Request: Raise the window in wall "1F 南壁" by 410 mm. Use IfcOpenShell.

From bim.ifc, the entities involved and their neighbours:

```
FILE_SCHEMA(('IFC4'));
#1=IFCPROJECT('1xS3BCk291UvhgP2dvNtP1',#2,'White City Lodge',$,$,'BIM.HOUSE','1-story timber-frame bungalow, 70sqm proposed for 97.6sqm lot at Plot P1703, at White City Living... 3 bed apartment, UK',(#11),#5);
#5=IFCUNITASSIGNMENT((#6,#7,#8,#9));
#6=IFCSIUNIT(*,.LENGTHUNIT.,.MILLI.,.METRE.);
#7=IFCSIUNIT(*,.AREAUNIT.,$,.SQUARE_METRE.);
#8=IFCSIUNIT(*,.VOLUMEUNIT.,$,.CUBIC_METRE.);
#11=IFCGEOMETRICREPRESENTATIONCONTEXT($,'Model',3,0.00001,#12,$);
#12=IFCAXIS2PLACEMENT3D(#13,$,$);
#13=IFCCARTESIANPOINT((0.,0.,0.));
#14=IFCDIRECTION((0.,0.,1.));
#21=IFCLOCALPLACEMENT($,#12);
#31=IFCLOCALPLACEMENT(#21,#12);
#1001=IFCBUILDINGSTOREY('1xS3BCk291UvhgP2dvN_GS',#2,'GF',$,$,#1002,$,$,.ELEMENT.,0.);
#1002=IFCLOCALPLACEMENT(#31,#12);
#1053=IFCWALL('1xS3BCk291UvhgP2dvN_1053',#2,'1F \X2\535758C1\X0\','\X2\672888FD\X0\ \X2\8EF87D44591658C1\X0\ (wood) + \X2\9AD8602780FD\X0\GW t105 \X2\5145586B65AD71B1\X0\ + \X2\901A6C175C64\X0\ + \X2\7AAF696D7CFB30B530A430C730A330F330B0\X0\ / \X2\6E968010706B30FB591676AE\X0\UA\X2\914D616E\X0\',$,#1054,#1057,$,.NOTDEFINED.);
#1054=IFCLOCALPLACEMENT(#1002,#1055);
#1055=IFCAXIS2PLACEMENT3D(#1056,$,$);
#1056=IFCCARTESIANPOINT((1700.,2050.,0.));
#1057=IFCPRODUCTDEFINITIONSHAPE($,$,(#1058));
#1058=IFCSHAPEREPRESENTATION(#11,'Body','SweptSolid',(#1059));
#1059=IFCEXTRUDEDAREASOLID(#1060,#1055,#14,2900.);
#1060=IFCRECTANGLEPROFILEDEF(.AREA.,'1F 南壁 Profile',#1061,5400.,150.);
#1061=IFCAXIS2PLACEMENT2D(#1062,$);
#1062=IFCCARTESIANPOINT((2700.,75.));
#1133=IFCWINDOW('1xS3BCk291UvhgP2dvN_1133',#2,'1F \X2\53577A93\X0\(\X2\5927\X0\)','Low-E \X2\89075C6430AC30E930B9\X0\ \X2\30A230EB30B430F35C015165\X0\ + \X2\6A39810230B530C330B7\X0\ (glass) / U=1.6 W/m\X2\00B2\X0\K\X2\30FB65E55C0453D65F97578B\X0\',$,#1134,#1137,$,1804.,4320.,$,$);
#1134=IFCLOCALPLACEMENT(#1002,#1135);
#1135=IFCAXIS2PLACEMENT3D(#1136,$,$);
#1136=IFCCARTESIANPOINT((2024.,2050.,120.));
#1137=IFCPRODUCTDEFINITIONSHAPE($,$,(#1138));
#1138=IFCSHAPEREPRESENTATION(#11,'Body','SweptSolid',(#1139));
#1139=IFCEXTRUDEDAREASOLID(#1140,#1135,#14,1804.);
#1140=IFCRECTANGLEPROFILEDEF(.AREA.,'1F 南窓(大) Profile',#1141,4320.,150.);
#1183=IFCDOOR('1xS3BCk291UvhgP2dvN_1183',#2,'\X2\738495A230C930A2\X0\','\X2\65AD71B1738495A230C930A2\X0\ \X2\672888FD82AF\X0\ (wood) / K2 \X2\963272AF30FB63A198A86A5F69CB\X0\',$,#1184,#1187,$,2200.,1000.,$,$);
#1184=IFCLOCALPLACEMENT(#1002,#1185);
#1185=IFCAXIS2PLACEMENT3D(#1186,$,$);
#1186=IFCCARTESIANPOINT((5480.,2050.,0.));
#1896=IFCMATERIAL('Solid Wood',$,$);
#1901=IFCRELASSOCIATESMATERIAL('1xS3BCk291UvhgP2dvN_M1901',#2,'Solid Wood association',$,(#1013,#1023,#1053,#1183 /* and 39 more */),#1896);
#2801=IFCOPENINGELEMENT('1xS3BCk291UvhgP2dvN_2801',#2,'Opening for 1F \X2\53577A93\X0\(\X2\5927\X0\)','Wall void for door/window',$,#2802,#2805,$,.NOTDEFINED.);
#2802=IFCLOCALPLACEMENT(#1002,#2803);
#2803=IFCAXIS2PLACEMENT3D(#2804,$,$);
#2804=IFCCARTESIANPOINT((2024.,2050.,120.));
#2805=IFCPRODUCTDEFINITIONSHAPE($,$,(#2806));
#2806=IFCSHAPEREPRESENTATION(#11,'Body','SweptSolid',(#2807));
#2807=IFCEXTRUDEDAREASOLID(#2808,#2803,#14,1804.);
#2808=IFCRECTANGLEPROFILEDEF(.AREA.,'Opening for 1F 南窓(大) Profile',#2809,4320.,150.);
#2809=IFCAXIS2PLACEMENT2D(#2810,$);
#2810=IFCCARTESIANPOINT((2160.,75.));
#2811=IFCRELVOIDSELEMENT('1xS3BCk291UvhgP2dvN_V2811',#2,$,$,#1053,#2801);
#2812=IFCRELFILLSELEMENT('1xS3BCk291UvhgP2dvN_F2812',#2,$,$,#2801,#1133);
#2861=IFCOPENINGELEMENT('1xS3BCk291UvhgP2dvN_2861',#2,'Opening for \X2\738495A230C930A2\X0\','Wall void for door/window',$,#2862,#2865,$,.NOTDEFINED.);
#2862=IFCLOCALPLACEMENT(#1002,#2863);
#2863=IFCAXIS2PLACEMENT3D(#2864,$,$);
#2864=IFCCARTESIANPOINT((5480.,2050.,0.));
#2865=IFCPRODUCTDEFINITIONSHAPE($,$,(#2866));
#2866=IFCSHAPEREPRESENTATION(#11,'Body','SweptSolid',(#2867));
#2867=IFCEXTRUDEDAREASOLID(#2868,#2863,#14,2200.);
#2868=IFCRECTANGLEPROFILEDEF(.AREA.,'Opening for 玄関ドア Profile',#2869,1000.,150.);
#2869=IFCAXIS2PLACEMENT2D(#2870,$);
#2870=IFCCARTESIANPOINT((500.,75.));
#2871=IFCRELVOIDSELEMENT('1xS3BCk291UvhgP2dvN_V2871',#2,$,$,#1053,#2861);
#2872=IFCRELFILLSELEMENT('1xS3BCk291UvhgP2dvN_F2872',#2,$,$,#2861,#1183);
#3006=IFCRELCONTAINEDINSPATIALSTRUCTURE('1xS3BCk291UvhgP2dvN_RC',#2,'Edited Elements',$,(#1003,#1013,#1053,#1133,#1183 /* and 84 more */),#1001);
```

```python
import numpy as np
import ifcopenshell
import ifcopenshell.api.geometry
import ifcopenshell.util.placement
import ifcopenshell.util.unit

model = ifcopenshell.open("bim.ifc")
unit_scale = ifcopenshell.util.unit.calculate_unit_scale(model)

window = model.by_guid("1xS3BCk291UvhgP2dvN_1133")
opening = window.FillsVoids[0].RelatingOpeningElement
dz = 410.0

shift = np.array([0.0, 0.0, dz])
# The window is not placed relative to its opening, so move both.
for product in (opening, window):
    matrix = ifcopenshell.util.placement.get_local_placement(product.ObjectPlacement)
    matrix[:3, 3] += shift
    ifcopenshell.api.geometry.edit_object_placement(model, product=product, matrix=matrix, is_si=False)

print(f"moved by {dz * unit_scale:+.3f} m")

model.write("bim_rev.ifc")
```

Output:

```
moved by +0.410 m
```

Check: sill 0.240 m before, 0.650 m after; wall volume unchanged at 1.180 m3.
